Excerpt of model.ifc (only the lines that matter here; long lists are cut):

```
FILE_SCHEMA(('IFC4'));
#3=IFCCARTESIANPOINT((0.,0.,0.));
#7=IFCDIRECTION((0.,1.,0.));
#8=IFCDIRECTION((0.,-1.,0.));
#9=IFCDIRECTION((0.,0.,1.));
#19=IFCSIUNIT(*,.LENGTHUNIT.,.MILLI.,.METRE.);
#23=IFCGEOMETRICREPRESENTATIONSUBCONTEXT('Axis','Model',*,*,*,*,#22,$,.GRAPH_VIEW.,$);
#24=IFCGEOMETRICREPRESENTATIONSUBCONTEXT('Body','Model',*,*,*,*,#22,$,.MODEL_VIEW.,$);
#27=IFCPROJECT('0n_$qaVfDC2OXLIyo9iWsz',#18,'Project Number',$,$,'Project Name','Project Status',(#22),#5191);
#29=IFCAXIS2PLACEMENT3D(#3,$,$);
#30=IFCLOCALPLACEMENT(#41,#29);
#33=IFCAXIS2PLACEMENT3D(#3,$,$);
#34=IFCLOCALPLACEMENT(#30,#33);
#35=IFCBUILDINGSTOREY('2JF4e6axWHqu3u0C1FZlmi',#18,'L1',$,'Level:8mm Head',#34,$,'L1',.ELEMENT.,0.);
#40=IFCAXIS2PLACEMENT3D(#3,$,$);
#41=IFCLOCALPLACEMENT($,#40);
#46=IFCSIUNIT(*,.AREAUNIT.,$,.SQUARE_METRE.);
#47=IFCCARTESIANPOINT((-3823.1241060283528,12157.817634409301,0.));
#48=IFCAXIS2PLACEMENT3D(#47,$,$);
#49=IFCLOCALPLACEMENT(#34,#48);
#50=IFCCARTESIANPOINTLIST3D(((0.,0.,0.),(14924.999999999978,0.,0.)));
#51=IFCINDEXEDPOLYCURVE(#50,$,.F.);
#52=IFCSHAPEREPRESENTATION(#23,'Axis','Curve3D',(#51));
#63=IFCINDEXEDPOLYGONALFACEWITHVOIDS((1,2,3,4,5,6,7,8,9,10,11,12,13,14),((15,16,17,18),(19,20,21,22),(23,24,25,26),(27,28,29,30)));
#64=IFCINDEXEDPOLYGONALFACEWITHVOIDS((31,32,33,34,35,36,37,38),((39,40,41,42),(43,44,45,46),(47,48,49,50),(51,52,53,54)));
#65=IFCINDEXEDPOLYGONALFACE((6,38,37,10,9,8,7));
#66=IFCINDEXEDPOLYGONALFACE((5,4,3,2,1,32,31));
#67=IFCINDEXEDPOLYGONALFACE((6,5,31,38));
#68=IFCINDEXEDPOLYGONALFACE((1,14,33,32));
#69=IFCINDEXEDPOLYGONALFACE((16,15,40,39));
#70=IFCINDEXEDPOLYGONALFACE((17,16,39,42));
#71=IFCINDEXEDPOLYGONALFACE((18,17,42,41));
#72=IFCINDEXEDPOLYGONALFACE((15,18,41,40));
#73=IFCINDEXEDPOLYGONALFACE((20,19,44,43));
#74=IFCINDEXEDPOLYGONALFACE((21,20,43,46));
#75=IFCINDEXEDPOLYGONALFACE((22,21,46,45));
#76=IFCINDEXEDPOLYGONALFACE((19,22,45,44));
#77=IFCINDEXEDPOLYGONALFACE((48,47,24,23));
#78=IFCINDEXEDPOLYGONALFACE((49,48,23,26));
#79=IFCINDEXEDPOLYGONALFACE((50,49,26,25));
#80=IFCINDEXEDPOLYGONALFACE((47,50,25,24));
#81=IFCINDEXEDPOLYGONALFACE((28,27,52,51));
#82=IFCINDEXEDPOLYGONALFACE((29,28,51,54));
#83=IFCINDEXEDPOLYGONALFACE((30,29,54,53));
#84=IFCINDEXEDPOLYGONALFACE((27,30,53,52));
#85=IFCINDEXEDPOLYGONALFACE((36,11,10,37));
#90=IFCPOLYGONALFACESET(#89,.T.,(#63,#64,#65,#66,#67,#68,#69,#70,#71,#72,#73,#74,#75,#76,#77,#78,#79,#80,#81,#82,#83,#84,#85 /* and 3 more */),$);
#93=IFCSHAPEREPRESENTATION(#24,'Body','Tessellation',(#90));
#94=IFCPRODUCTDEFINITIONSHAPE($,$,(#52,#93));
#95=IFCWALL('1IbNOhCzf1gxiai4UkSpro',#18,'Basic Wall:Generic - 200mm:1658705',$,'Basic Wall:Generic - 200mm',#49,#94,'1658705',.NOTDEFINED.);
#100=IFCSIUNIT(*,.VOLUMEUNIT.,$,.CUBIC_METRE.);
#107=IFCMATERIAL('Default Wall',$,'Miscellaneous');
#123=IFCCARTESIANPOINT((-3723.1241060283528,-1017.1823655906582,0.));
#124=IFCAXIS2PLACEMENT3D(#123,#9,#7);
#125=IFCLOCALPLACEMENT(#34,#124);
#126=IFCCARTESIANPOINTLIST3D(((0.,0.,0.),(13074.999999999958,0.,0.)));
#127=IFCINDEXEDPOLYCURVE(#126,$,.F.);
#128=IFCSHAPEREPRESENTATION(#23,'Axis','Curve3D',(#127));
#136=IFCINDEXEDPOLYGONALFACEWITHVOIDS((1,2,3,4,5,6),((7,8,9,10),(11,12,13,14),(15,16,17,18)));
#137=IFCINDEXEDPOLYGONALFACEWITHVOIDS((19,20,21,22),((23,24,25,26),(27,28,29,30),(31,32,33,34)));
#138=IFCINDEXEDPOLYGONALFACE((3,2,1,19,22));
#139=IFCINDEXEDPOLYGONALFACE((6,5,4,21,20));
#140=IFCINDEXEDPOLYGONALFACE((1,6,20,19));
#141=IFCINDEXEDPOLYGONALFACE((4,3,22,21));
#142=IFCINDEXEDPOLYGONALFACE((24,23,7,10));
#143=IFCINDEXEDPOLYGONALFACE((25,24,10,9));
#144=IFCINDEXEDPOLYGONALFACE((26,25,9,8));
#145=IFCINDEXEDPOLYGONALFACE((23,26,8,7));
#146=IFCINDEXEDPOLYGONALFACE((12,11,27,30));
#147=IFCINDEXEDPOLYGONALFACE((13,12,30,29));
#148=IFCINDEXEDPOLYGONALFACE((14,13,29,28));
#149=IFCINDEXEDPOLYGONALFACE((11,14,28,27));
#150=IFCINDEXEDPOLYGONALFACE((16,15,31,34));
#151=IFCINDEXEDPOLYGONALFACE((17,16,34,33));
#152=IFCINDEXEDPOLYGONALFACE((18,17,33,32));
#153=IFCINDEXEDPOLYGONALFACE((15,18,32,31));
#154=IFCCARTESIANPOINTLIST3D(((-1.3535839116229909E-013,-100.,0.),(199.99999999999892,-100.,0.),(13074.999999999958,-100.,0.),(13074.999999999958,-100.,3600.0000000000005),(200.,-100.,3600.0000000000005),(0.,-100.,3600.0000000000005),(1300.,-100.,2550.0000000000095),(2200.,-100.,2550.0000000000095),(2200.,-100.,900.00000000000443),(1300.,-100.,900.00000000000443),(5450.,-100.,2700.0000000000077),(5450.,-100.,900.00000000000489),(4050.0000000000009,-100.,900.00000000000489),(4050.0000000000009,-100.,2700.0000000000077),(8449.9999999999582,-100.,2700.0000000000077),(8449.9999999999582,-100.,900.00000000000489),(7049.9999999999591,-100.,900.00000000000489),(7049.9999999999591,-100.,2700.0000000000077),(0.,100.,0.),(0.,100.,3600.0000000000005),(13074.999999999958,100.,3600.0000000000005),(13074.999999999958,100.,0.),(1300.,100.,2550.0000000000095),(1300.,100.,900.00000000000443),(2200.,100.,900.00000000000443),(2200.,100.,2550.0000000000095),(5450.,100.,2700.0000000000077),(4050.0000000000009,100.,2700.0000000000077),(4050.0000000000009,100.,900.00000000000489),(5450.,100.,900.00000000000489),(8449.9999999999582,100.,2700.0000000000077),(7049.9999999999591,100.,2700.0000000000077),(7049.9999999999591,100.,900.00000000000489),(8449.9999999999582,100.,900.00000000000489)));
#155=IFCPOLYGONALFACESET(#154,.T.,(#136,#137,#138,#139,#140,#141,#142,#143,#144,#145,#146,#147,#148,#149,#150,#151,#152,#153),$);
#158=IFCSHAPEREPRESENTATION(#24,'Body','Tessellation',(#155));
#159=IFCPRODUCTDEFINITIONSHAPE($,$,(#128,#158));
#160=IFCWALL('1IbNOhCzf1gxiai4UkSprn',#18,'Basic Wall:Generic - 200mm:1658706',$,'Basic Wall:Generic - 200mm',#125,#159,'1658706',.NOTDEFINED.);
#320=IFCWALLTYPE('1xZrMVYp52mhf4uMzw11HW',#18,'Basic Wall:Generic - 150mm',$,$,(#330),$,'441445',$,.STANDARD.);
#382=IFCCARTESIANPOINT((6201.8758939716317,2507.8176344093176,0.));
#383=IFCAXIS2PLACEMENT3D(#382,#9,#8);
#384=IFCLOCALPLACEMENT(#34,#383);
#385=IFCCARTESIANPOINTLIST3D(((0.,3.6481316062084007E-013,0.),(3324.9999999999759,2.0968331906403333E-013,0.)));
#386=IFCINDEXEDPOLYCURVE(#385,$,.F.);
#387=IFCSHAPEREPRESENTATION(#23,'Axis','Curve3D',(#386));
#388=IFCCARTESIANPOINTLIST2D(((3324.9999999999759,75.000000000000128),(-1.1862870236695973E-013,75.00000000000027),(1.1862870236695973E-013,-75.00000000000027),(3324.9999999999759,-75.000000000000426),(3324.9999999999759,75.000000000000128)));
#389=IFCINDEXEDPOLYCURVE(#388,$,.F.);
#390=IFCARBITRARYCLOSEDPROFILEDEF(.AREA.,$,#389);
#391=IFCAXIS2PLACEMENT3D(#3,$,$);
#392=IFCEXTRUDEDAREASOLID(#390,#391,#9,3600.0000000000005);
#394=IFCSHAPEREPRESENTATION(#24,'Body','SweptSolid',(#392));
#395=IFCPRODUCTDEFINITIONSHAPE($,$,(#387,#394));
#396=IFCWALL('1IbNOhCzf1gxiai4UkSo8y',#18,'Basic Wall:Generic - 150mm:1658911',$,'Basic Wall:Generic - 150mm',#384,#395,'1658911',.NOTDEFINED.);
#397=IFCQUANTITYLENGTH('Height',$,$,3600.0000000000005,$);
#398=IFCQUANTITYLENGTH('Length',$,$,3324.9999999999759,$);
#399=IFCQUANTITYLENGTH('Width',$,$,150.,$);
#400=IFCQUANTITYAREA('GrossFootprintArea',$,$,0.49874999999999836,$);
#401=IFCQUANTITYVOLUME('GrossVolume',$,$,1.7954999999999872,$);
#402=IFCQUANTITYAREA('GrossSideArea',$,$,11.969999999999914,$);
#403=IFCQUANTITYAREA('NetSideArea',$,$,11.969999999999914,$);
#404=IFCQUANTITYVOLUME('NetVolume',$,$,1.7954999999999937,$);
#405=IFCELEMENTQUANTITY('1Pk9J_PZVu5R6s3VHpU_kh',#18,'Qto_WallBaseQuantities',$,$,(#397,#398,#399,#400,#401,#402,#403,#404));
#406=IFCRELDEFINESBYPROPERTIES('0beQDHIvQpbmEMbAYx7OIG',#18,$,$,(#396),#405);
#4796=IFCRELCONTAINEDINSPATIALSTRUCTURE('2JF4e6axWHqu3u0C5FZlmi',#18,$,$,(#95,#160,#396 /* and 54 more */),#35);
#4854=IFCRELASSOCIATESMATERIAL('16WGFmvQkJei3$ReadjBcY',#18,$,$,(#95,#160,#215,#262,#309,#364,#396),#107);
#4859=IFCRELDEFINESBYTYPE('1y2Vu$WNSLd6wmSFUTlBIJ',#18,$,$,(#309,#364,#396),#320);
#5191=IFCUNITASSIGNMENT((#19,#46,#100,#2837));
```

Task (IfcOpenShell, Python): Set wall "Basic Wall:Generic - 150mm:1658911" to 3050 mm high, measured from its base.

```python
import ifcopenshell
import ifcopenshell.api.pset
import ifcopenshell.geom
import ifcopenshell.util.element
import ifcopenshell.util.representation
import ifcopenshell.util.shape
import ifcopenshell.util.unit

model = ifcopenshell.open("model.ifc")
unit_scale = ifcopenshell.util.unit.calculate_unit_scale(model)
area_scale = ifcopenshell.util.unit.calculate_unit_scale(model, "AREAUNIT")
volume_scale = ifcopenshell.util.unit.calculate_unit_scale(model, "VOLUMEUNIT")
settings = ifcopenshell.geom.settings()


def volume(element):
    """Net volume in cubic metres, openings subtracted."""
    shape = ifcopenshell.geom.create_shape(settings, element)
    return ifcopenshell.util.shape.get_volume(shape.geometry)


wall = model.by_guid("1IbNOhCzf1gxiai4UkSo8y")
before = volume(wall)

body = ifcopenshell.util.representation.get_representation(wall, "Model", "Body")
solid = body.Items[0]
old_height = solid.Depth
solid.Depth = 3.05 / unit_scale
after = volume(wall)
thickness = 0.15  # wall thickness in metres

# Update the stored height, areas and volumes.
qto = model.by_id(ifcopenshell.util.element.get_pset(wall, "Qto_WallBaseQuantities", should_inherit=False)["id"])
ifcopenshell.api.pset.edit_qto(model, qto=qto, properties={
    "Height": solid.Depth,
    "GrossVolume": ifcopenshell.util.element.get_pset(wall, "Qto_WallBaseQuantities", "GrossVolume") * solid.Depth / old_height,
    "GrossSideArea": ifcopenshell.util.element.get_pset(wall, "Qto_WallBaseQuantities", "GrossSideArea") * solid.Depth / old_height,
    "NetSideArea": after / thickness / area_scale,
    "NetVolume": after / volume_scale,
})

print(f"height {old_height:g} -> {solid.Depth:g}, volume {before:.3f} -> {after:.3f} m3")

model.write("model_edited.ifc")
```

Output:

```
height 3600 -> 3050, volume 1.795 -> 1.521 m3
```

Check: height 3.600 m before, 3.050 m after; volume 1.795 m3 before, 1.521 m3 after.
